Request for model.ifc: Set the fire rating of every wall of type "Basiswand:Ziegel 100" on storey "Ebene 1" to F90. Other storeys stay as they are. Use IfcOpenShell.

First a look at what the model holds.

```python
import ifcopenshell
import ifcopenshell.util.element

model = ifcopenshell.open("model.ifc")
print(model.schema)
storey = next(s for s in model.by_type("IfcBuildingStorey") if s.Name == "Ebene 1")
walls = [e for e in ifcopenshell.util.element.get_decomposition(storey) if e.is_a("IfcWall")]
seen = {}
for e in walls:
    element_type = ifcopenshell.util.element.get_type(e)
    key = (element_type.Name if element_type != e and element_type else None, ifcopenshell.util.element.get_pset(e, "Pset_WallCommon", "FireRating"))
    seen[key] = seen.get(key, 0) + 1
for (name, value), count in sorted(seen.items(), key=str):
    print(count, "x", name, "|", value)
```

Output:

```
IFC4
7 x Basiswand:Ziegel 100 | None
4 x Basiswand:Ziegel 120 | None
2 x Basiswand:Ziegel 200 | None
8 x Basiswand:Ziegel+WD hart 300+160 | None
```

```python
import ifcopenshell
import ifcopenshell.api.pset
import ifcopenshell.util.element

model = ifcopenshell.open("model.ifc")

storey = next(s for s in model.by_type("IfcBuildingStorey") if s.Name == "Ebene 1")
walls = [e for e in ifcopenshell.util.element.get_decomposition(storey) if e.is_a("IfcWall")]

count = 0
for e in walls:
    element_type = ifcopenshell.util.element.get_type(e)
    if element_type in (None, e) or element_type.Name != "Basiswand:Ziegel 100":
        continue
    # add_pset returns the element's existing set when there is one.
    pset = ifcopenshell.api.pset.add_pset(model, product=e, name="Pset_WallCommon")
    ifcopenshell.api.pset.edit_pset(model, pset=pset, properties={"FireRating": "F90"})
    count += 1

print(count, "walls updated")

model.write("model_rev.ifc")
```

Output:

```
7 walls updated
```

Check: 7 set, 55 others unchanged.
